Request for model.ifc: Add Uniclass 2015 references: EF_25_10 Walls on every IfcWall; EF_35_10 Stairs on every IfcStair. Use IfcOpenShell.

First a look at what the model holds.

```python
import ifcopenshell

model = ifcopenshell.open("model.ifc")
print(model.schema)
print("classifications:", [c.Name for c in model.by_type("IfcClassification")])
for ifc_class in ("IfcDoor", "IfcRoof", "IfcStair", "IfcWall", "IfcWindow"):
    print(ifc_class, len(model.by_type(ifc_class)))
```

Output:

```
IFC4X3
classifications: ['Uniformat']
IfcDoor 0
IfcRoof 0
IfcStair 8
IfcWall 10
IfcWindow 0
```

```python
import ifcopenshell
import ifcopenshell.api.classification

model = ifcopenshell.open("model.ifc")

system = ifcopenshell.api.classification.add_classification(model, classification="Uniclass 2015")

codes = {
    "IfcWall": ("EF_25_10", "Walls"),
    "IfcStair": ("EF_35_10", "Stairs"),
}
for ifc_class, (code, name) in codes.items():
    products = model.by_type(ifc_class)
    ifcopenshell.api.classification.add_reference(
        model, products=products, classification=system, identification=code, name=name
    )
    print(code, len(products))

model.write("model_edited.ifc")
```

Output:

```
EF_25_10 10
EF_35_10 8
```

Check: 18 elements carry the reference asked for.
